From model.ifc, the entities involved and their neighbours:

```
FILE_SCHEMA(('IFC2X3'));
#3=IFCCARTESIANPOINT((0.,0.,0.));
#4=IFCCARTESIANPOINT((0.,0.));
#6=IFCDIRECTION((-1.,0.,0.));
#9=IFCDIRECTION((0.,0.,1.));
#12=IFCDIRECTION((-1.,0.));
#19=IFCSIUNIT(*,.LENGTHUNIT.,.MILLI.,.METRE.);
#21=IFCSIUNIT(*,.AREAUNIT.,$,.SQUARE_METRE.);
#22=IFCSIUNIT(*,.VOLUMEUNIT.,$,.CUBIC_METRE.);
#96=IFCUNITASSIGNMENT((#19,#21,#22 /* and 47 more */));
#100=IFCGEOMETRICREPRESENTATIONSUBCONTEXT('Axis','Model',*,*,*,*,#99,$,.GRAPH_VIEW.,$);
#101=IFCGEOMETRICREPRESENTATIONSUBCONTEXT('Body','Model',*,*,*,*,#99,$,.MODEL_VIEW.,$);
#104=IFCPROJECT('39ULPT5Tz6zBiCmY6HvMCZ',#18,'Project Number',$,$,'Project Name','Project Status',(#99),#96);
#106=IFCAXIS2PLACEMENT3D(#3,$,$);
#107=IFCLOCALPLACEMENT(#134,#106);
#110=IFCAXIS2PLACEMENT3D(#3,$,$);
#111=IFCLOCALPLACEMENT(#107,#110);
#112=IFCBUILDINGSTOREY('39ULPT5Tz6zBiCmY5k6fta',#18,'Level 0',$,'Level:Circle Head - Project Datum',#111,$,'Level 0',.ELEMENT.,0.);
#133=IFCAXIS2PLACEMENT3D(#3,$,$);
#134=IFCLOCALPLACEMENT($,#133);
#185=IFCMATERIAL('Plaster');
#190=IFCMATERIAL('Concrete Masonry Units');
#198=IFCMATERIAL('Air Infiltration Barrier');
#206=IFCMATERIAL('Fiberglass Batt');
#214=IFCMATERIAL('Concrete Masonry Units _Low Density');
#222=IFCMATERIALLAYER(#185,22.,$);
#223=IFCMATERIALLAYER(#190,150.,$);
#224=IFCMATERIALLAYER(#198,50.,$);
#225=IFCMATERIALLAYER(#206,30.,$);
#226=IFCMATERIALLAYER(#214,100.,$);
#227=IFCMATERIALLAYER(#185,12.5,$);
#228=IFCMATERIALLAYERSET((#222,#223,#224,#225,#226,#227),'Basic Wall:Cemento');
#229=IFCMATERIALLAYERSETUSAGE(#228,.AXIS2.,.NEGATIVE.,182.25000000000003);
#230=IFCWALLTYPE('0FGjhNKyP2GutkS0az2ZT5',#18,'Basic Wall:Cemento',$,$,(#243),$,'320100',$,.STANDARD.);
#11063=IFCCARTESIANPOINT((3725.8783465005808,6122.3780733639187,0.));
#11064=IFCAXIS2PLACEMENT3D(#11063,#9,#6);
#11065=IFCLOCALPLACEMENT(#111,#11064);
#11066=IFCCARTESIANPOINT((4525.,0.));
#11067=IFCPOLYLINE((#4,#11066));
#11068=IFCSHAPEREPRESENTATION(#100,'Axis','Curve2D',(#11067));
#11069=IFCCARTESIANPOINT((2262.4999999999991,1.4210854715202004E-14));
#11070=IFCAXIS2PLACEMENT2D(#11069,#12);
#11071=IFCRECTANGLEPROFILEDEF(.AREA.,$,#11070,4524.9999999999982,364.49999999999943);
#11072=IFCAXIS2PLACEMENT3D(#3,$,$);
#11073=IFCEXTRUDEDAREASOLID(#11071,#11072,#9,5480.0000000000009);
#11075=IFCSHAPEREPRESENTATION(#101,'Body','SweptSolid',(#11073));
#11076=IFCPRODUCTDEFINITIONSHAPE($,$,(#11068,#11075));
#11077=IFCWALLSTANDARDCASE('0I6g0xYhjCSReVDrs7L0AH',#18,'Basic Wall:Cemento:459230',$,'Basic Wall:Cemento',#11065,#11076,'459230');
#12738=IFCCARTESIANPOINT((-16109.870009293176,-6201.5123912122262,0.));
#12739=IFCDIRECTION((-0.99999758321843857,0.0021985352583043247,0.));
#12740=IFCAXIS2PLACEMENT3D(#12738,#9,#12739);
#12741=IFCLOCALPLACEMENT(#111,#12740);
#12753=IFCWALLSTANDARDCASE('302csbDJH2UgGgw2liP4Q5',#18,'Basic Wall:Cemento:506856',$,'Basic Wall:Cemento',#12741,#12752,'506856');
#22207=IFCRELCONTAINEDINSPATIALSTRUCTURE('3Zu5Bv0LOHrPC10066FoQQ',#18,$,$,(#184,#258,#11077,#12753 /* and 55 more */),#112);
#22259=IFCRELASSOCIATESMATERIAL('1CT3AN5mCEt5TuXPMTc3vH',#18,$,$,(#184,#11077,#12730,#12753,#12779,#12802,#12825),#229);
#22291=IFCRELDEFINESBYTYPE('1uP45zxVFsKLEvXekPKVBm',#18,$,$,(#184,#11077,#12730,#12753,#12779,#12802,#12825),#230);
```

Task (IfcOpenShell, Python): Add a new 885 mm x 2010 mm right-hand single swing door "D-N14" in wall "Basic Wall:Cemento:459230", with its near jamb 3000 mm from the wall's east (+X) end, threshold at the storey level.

```python
import numpy as np
import ifcopenshell
import ifcopenshell.api.feature
import ifcopenshell.api.geometry
import ifcopenshell.api.root
import ifcopenshell.api.spatial
import ifcopenshell.api.type
import ifcopenshell.geom
import ifcopenshell.util.element
import ifcopenshell.util.placement
import ifcopenshell.util.representation
import ifcopenshell.util.shape
import ifcopenshell.util.unit

model = ifcopenshell.open("model.ifc")
unit_scale = ifcopenshell.util.unit.calculate_unit_scale(model)
settings = ifcopenshell.geom.settings()


def volume(element):
    """Net volume in cubic metres, openings subtracted."""
    shape = ifcopenshell.geom.create_shape(settings, element)
    return ifcopenshell.util.shape.get_volume(shape.geometry)


wall = model.by_guid("0I6g0xYhjCSReVDrs7L0AH")
storey = ifcopenshell.util.element.get_container(wall, ifc_class="IfcBuildingStorey")
context = ifcopenshell.util.representation.get_context(model, "Model", "Body", "MODEL_VIEW")
before = volume(wall)

width, height, from_end, sill = 0.885, 2.01, 3, 0.0  # metres

# The wall runs along its own X axis, and the end named is its -X end.
wall_shape = ifcopenshell.geom.create_shape(settings, wall)
x, y, z = ifcopenshell.util.shape.get_vertices(wall_shape.geometry).T
start = x.min() + from_end
face, thickness = float(y.min()), float(y.max() - y.min())
wall_matrix = ifcopenshell.util.placement.get_local_placement(wall.ObjectPlacement)
level = ifcopenshell.util.placement.get_local_placement(storey.ObjectPlacement)[2, 3]


def in_wall(x, y):
    """Placement at x, y metres in the wall's axes, at sill height."""
    matrix = wall_matrix.copy()
    matrix[:, 3] = wall_matrix @ np.array([x / unit_scale, y / unit_scale, 0.0, 1.0])
    matrix[2, 3] = level + sill / unit_scale
    return matrix


# Opening: a box that overshoots both wall faces by 50 mm.
opening = ifcopenshell.api.root.create_entity(model, ifc_class="IfcOpeningElement")
box = ifcopenshell.api.geometry.add_wall_representation(
    model, context=context, length=width, height=height, thickness=thickness + 0.1
)
ifcopenshell.api.geometry.assign_representation(model, product=opening, representation=box)
ifcopenshell.api.geometry.edit_object_placement(model, product=opening, matrix=in_wall(start, face - 0.05), is_si=False)
ifcopenshell.api.feature.add_feature(model, feature=opening, element=wall)

door = ifcopenshell.api.root.create_entity(model, ifc_class="IfcDoor", name="D-N14")
door.OverallWidth, door.OverallHeight = width / unit_scale, height / unit_scale
body = ifcopenshell.api.geometry.add_door_representation(
    model,
    context=context,
    overall_width=door.OverallWidth,
    overall_height=door.OverallHeight,
    operation_type="SINGLE_SWING_RIGHT",
    lining_properties={"LiningDepth": thickness / unit_scale, "ThresholdDepth": thickness / unit_scale},
)
ifcopenshell.api.geometry.assign_representation(model, product=door, representation=body)
ifcopenshell.api.spatial.assign_container(model, products=[door], relating_structure=storey)
fills = ifcopenshell.api.feature.add_filling(model, opening=opening, element=door)
fills.OwnerHistory = door.OwnerHistory  # required in IFC2X3

# IFC2X3 keeps the operation on the door style.
style = ifcopenshell.api.root.create_entity(model, ifc_class="IfcDoorStyle", name="D-N14")
style.OperationType, style.ConstructionType = "SINGLE_SWING_RIGHT", "NOTDEFINED"
style.ParameterTakesPrecedence = style.Sizeable = False
ifcopenshell.api.type.assign_type(model, related_objects=[door], relating_type=style)

# The lining spans the wall, so the door starts at the wall face.
ifcopenshell.api.geometry.edit_object_placement(model, product=door, matrix=in_wall(start, face), is_si=False)

after = volume(wall)

print(f"wall volume {before:.3f} -> {after:.3f} m3")

model.write("model_edited.ifc")
```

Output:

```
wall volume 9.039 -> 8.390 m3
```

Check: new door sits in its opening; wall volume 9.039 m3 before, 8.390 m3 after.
